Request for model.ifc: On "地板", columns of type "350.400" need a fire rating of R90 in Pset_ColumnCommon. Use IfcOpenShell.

First a look at what the model holds.

```python
import ifcopenshell
import ifcopenshell.util.element

model = ifcopenshell.open("model.ifc")
print(model.schema)
storey = next(s for s in model.by_type("IfcBuildingStorey") if s.Name == "地板")
columns = [e for e in ifcopenshell.util.element.get_decomposition(storey) if e.is_a("IfcColumn")]
seen = {}
for e in columns:
    element_type = ifcopenshell.util.element.get_type(e)
    key = (element_type.Name if element_type != e and element_type else None, ifcopenshell.util.element.get_pset(e, "Pset_ColumnCommon", "FireRating"))
    seen[key] = seen.get(key, 0) + 1
for (name, value), count in sorted(seen.items(), key=str):
    print(count, "x", name, "|", value)
```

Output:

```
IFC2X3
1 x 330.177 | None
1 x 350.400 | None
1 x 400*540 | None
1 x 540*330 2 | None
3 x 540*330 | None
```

```python
import ifcopenshell
import ifcopenshell.api.pset
import ifcopenshell.util.element

model = ifcopenshell.open("model.ifc")

storey = next(s for s in model.by_type("IfcBuildingStorey") if s.Name == "地板")
columns = [e for e in ifcopenshell.util.element.get_decomposition(storey) if e.is_a("IfcColumn")]

count = 0
for e in columns:
    element_type = ifcopenshell.util.element.get_type(e)
    if element_type in (None, e) or element_type.Name != "350.400":
        continue
    # add_pset returns the element's existing set when there is one.
    pset = ifcopenshell.api.pset.add_pset(model, product=e, name="Pset_ColumnCommon")
    ifcopenshell.api.pset.edit_pset(model, pset=pset, properties={"FireRating": "R90"})
    count += 1

print(count, "columns updated")

model.write("model_v2.ifc")
```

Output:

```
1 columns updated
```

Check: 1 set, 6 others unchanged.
